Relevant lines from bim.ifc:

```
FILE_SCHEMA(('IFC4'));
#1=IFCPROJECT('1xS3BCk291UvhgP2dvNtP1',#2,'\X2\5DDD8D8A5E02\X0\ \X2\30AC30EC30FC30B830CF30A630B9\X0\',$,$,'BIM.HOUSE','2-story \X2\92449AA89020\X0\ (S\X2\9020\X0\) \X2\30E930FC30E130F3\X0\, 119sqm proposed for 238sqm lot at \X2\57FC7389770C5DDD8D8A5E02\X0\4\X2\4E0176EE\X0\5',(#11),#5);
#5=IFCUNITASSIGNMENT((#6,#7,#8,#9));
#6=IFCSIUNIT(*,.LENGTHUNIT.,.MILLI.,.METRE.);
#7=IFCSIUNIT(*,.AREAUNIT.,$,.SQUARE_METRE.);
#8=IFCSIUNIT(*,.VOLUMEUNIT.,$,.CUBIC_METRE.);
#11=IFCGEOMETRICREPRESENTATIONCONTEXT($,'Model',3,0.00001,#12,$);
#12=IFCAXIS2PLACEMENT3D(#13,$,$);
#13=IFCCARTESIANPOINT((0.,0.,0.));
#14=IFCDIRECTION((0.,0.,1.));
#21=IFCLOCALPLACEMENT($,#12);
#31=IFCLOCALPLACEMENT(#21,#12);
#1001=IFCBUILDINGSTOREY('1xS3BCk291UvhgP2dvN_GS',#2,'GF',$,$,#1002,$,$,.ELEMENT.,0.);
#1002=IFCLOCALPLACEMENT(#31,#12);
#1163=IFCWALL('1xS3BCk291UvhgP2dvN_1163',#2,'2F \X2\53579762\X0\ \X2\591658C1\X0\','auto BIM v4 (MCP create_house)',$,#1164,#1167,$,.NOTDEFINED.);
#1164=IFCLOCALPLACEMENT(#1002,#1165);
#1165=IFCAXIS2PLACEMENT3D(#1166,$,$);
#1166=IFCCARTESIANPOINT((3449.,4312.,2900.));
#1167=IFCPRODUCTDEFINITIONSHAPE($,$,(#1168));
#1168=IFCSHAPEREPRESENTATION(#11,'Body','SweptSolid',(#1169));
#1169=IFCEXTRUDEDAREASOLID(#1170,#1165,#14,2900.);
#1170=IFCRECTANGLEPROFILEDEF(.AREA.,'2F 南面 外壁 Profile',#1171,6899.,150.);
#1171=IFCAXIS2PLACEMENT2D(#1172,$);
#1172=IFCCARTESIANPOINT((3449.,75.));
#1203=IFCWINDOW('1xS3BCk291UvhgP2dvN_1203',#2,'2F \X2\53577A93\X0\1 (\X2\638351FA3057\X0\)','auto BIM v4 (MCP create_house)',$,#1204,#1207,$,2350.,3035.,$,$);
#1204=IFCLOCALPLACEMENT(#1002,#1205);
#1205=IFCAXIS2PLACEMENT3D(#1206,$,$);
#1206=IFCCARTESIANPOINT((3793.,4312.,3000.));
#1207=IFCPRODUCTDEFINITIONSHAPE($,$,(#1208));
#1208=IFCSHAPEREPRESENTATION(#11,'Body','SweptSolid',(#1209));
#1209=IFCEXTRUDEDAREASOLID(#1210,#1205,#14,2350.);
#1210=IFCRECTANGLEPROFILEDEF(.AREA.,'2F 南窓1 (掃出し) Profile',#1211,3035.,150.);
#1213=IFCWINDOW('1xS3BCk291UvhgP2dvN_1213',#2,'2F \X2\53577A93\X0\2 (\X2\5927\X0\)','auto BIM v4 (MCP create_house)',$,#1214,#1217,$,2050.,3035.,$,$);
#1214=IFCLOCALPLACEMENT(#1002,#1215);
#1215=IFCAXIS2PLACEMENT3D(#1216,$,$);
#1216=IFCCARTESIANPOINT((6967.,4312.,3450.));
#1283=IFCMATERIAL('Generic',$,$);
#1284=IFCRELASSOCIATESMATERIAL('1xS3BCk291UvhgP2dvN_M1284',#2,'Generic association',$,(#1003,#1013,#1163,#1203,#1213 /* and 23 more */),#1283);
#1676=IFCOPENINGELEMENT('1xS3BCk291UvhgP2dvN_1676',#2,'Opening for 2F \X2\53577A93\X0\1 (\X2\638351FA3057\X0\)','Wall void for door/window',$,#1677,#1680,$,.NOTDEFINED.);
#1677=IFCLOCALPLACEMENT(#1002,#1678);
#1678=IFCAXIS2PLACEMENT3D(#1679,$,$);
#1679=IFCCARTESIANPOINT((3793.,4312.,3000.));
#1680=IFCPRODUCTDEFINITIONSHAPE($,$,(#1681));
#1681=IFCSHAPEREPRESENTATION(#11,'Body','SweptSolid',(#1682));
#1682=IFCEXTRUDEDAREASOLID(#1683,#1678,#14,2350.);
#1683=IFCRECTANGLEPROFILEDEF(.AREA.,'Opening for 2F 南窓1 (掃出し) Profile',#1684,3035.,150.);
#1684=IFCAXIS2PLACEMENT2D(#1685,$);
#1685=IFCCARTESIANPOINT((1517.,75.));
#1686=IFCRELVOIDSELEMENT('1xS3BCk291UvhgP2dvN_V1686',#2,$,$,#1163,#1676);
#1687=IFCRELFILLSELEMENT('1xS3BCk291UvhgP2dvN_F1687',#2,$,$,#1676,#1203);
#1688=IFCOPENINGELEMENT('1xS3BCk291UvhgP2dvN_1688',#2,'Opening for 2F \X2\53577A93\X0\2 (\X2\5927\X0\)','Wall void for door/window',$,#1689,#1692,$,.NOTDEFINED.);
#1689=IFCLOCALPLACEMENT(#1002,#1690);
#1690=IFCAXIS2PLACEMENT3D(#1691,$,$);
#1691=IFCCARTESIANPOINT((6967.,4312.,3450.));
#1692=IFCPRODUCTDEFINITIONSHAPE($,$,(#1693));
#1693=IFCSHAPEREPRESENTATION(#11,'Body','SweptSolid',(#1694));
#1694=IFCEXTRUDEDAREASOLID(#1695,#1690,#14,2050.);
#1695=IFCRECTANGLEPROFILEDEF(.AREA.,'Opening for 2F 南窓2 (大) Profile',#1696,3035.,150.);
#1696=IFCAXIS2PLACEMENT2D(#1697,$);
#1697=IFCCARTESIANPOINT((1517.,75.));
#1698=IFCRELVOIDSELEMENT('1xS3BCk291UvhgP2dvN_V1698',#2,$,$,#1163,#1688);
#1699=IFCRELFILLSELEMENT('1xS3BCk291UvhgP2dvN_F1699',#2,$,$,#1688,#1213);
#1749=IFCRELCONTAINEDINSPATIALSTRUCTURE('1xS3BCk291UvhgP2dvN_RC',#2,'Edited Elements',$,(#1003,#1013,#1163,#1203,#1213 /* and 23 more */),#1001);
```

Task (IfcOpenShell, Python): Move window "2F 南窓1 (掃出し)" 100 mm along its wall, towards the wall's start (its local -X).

```python
import ifcopenshell
import ifcopenshell.api.geometry
import ifcopenshell.util.placement
import ifcopenshell.util.unit

model = ifcopenshell.open("bim.ifc")
unit_scale = ifcopenshell.util.unit.calculate_unit_scale(model)

window = model.by_id(1203)
opening = window.FillsVoids[0].RelatingOpeningElement
wall = opening.VoidsElements[0].RelatingBuildingElement

wall_matrix = ifcopenshell.util.placement.get_local_placement(wall.ObjectPlacement)
shift = wall_matrix[:3, 0] * -0.1 / unit_scale
before = ifcopenshell.util.placement.get_local_placement(window.ObjectPlacement)[:3, 3].copy()

# The window is not placed relative to its opening, so move both.
for product in (opening, window):
    matrix = ifcopenshell.util.placement.get_local_placement(product.ObjectPlacement)
    matrix[:3, 3] += shift
    ifcopenshell.api.geometry.edit_object_placement(model, product=product, matrix=matrix, is_si=False)

after = ifcopenshell.util.placement.get_local_placement(window.ObjectPlacement)[:3, 3]
print("window moved by", (after - before).round(3) + 0.0)

model.write("bim-out.ifc")
```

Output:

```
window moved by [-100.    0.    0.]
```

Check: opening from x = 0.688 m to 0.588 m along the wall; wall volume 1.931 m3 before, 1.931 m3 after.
